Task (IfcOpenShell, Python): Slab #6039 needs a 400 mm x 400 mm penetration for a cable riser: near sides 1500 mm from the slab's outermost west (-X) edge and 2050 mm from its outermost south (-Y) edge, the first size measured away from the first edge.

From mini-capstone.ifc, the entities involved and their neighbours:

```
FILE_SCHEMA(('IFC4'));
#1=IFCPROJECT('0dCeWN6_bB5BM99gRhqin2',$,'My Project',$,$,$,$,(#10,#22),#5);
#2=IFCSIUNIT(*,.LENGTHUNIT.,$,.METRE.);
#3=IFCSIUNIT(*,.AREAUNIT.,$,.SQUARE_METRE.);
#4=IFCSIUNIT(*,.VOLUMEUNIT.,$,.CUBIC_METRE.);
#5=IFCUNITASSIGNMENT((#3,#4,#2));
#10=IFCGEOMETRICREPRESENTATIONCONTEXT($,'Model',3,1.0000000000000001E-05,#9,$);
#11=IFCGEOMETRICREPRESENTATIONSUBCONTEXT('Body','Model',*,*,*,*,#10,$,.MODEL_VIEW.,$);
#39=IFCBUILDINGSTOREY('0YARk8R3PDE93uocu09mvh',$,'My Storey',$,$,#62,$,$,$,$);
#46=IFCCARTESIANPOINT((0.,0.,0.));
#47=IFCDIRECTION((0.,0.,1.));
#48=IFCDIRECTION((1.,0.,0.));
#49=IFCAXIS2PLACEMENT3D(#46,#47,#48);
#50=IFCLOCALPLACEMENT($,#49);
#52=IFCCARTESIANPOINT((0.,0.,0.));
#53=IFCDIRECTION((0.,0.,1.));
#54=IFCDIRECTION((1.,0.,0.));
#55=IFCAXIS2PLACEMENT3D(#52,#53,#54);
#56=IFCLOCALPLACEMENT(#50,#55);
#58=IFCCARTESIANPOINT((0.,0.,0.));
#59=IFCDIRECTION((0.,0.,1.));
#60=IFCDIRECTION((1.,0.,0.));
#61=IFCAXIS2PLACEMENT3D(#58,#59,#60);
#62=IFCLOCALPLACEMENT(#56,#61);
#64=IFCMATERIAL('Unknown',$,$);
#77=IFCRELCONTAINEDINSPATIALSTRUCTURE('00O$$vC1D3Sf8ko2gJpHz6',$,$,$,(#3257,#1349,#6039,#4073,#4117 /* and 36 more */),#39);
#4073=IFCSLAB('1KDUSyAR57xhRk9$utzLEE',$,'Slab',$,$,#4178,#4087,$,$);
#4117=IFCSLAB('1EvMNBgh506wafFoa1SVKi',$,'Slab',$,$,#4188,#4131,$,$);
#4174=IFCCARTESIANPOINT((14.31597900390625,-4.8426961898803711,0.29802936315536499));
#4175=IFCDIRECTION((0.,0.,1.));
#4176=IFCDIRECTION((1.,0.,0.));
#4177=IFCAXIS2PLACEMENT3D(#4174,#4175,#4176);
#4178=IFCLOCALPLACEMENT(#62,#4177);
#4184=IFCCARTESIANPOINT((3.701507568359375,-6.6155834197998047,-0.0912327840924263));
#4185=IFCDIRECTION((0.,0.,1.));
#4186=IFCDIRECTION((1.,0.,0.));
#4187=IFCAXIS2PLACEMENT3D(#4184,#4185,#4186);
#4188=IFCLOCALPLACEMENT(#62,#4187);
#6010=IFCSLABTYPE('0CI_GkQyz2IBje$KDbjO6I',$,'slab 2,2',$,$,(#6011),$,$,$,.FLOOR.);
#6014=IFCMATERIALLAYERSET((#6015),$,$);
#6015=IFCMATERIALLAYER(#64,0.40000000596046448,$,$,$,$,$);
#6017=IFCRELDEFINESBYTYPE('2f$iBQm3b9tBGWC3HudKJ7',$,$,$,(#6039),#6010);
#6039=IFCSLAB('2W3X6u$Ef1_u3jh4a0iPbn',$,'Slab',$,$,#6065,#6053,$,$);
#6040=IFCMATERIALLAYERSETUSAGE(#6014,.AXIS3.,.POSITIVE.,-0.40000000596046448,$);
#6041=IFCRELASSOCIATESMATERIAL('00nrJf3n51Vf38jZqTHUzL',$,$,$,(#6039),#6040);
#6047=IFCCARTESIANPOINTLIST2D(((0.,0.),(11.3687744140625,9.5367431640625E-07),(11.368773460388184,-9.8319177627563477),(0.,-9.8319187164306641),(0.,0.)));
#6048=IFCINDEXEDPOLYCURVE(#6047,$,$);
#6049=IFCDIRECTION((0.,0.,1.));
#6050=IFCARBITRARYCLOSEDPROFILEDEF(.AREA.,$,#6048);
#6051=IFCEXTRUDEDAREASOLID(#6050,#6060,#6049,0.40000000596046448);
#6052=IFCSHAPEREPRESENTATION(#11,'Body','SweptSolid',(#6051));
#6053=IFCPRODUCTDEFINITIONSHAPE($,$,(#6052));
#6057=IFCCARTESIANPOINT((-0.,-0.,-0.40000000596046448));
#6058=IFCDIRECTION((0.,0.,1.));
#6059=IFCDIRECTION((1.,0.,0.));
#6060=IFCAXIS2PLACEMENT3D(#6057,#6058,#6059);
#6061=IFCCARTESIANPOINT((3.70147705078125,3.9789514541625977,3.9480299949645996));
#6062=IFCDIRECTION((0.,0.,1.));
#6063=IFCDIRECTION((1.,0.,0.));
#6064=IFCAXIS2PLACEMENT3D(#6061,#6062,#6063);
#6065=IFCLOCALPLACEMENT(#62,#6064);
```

```python
import numpy as np
import ifcopenshell
import ifcopenshell.api.feature
import ifcopenshell.api.geometry
import ifcopenshell.api.root
import ifcopenshell.geom
import ifcopenshell.util.placement
import ifcopenshell.util.representation
import ifcopenshell.util.shape
import ifcopenshell.util.unit

model = ifcopenshell.open("mini-capstone.ifc")
unit_scale = ifcopenshell.util.unit.calculate_unit_scale(model)
settings = ifcopenshell.geom.settings()


def volume(element):
    """Net volume in cubic metres, openings subtracted."""
    shape = ifcopenshell.geom.create_shape(settings, element)
    return ifcopenshell.util.shape.get_volume(shape.geometry)


slab = model.by_guid("2W3X6u$Ef1_u3jh4a0iPbn")
before = volume(slab)

# Extent in the slab's own axes, in metres. The edges named are its -X and -Y sides.
slab_shape = ifcopenshell.geom.create_shape(settings, slab)
vertices = ifcopenshell.util.shape.get_vertices(slab_shape.geometry)
x_min, y_min, bottom = vertices.min(axis=0)
top = vertices[:, 2].max()

opening = ifcopenshell.api.root.create_entity(model, ifc_class="IfcOpeningElement", name="Cable riser opening", predefined_type="OPENING")
context = ifcopenshell.util.representation.get_context(model, "Model", "Body", "MODEL_VIEW")
width, depth = 0.4, 0.4
outline = [(0.0, 0.0), (width, 0.0), (width, depth), (0.0, depth), (0.0, 0.0)]
# Overshoot both faces by 50 mm so the cut is clean.
shape = ifcopenshell.api.geometry.add_slab_representation(
    model, context=context, depth=top - bottom + 0.1, polyline=outline
)
ifcopenshell.api.geometry.assign_representation(model, product=opening, representation=shape)

matrix = ifcopenshell.util.placement.get_local_placement(slab.ObjectPlacement)
matrix[:, 3] = matrix @ np.append(np.array([x_min + 1.5, y_min + 2.05, bottom - 0.05]) / unit_scale, 1.0)
ifcopenshell.api.geometry.edit_object_placement(model, product=opening, matrix=matrix, is_si=False)
ifcopenshell.api.feature.add_feature(model, feature=opening, element=slab)

after = volume(slab)

print(f"slab volume {before:.3f} -> {after:.3f} m3")

model.write("mini-capstone_edited.ifc")
```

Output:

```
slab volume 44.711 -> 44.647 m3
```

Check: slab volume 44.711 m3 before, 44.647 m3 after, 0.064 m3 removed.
